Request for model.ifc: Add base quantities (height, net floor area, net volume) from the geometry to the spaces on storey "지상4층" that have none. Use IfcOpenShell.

First a look at what the model holds.

```python
import ifcopenshell
import ifcopenshell.util.element
import ifcopenshell.util.unit

model = ifcopenshell.open("model.ifc")
print(model.schema)
for unit_type in ("LENGTHUNIT", "AREAUNIT", "VOLUMEUNIT"):
    print(unit_type, ifcopenshell.util.unit.calculate_unit_scale(model, unit_type))
storey = next(s for s in model.by_type("IfcBuildingStorey") if s.Name == "지상4층")
spaces = [e for e in ifcopenshell.util.element.get_decomposition(storey) if e.is_a("IfcSpace")]
for e in sorted(spaces, key=lambda e: e.id()):
    print(e.id(), e.is_a(), e.Name, list(ifcopenshell.util.element.get_psets(e, qtos_only=True)), sep=" | ")
```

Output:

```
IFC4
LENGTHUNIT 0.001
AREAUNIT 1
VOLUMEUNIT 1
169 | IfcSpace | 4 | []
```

```python
import ifcopenshell
import ifcopenshell.api.pset
import ifcopenshell.geom
import ifcopenshell.util.element
import ifcopenshell.util.shape
import ifcopenshell.util.unit

model = ifcopenshell.open("model.ifc")
unit_scale = ifcopenshell.util.unit.calculate_unit_scale(model)
area_scale = ifcopenshell.util.unit.calculate_unit_scale(model, "AREAUNIT")
volume_scale = ifcopenshell.util.unit.calculate_unit_scale(model, "VOLUMEUNIT")
settings = ifcopenshell.geom.settings()

storey = next(s for s in model.by_type("IfcBuildingStorey") if s.Name == "지상4층")
spaces = [e for e in ifcopenshell.util.element.get_decomposition(storey) if e.is_a("IfcSpace")]

for e in sorted(spaces, key=lambda e: e.id()):
    if ifcopenshell.util.element.get_psets(e, qtos_only=True, should_inherit=False):
        continue
    # Geometry comes back in metres, in the element's own axes.
    shape = ifcopenshell.geom.create_shape(settings, e)
    values = {
        "Height": ifcopenshell.util.shape.get_z(shape.geometry) / unit_scale,
        "NetFloorArea": ifcopenshell.util.shape.get_footprint_area(shape.geometry) / area_scale,
        "NetVolume": ifcopenshell.util.shape.get_volume(shape.geometry) / volume_scale,
    }
    qto = ifcopenshell.api.pset.add_qto(model, product=e, name="Qto_SpaceBaseQuantities")
    ifcopenshell.api.pset.edit_qto(model, qto=qto, properties=values)
    print(e.id(), {k: round(v, 3) for k, v in values.items()})

model.write("model-out.ifc")
```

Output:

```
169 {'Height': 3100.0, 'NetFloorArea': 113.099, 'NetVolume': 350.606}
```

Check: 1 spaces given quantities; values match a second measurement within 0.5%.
